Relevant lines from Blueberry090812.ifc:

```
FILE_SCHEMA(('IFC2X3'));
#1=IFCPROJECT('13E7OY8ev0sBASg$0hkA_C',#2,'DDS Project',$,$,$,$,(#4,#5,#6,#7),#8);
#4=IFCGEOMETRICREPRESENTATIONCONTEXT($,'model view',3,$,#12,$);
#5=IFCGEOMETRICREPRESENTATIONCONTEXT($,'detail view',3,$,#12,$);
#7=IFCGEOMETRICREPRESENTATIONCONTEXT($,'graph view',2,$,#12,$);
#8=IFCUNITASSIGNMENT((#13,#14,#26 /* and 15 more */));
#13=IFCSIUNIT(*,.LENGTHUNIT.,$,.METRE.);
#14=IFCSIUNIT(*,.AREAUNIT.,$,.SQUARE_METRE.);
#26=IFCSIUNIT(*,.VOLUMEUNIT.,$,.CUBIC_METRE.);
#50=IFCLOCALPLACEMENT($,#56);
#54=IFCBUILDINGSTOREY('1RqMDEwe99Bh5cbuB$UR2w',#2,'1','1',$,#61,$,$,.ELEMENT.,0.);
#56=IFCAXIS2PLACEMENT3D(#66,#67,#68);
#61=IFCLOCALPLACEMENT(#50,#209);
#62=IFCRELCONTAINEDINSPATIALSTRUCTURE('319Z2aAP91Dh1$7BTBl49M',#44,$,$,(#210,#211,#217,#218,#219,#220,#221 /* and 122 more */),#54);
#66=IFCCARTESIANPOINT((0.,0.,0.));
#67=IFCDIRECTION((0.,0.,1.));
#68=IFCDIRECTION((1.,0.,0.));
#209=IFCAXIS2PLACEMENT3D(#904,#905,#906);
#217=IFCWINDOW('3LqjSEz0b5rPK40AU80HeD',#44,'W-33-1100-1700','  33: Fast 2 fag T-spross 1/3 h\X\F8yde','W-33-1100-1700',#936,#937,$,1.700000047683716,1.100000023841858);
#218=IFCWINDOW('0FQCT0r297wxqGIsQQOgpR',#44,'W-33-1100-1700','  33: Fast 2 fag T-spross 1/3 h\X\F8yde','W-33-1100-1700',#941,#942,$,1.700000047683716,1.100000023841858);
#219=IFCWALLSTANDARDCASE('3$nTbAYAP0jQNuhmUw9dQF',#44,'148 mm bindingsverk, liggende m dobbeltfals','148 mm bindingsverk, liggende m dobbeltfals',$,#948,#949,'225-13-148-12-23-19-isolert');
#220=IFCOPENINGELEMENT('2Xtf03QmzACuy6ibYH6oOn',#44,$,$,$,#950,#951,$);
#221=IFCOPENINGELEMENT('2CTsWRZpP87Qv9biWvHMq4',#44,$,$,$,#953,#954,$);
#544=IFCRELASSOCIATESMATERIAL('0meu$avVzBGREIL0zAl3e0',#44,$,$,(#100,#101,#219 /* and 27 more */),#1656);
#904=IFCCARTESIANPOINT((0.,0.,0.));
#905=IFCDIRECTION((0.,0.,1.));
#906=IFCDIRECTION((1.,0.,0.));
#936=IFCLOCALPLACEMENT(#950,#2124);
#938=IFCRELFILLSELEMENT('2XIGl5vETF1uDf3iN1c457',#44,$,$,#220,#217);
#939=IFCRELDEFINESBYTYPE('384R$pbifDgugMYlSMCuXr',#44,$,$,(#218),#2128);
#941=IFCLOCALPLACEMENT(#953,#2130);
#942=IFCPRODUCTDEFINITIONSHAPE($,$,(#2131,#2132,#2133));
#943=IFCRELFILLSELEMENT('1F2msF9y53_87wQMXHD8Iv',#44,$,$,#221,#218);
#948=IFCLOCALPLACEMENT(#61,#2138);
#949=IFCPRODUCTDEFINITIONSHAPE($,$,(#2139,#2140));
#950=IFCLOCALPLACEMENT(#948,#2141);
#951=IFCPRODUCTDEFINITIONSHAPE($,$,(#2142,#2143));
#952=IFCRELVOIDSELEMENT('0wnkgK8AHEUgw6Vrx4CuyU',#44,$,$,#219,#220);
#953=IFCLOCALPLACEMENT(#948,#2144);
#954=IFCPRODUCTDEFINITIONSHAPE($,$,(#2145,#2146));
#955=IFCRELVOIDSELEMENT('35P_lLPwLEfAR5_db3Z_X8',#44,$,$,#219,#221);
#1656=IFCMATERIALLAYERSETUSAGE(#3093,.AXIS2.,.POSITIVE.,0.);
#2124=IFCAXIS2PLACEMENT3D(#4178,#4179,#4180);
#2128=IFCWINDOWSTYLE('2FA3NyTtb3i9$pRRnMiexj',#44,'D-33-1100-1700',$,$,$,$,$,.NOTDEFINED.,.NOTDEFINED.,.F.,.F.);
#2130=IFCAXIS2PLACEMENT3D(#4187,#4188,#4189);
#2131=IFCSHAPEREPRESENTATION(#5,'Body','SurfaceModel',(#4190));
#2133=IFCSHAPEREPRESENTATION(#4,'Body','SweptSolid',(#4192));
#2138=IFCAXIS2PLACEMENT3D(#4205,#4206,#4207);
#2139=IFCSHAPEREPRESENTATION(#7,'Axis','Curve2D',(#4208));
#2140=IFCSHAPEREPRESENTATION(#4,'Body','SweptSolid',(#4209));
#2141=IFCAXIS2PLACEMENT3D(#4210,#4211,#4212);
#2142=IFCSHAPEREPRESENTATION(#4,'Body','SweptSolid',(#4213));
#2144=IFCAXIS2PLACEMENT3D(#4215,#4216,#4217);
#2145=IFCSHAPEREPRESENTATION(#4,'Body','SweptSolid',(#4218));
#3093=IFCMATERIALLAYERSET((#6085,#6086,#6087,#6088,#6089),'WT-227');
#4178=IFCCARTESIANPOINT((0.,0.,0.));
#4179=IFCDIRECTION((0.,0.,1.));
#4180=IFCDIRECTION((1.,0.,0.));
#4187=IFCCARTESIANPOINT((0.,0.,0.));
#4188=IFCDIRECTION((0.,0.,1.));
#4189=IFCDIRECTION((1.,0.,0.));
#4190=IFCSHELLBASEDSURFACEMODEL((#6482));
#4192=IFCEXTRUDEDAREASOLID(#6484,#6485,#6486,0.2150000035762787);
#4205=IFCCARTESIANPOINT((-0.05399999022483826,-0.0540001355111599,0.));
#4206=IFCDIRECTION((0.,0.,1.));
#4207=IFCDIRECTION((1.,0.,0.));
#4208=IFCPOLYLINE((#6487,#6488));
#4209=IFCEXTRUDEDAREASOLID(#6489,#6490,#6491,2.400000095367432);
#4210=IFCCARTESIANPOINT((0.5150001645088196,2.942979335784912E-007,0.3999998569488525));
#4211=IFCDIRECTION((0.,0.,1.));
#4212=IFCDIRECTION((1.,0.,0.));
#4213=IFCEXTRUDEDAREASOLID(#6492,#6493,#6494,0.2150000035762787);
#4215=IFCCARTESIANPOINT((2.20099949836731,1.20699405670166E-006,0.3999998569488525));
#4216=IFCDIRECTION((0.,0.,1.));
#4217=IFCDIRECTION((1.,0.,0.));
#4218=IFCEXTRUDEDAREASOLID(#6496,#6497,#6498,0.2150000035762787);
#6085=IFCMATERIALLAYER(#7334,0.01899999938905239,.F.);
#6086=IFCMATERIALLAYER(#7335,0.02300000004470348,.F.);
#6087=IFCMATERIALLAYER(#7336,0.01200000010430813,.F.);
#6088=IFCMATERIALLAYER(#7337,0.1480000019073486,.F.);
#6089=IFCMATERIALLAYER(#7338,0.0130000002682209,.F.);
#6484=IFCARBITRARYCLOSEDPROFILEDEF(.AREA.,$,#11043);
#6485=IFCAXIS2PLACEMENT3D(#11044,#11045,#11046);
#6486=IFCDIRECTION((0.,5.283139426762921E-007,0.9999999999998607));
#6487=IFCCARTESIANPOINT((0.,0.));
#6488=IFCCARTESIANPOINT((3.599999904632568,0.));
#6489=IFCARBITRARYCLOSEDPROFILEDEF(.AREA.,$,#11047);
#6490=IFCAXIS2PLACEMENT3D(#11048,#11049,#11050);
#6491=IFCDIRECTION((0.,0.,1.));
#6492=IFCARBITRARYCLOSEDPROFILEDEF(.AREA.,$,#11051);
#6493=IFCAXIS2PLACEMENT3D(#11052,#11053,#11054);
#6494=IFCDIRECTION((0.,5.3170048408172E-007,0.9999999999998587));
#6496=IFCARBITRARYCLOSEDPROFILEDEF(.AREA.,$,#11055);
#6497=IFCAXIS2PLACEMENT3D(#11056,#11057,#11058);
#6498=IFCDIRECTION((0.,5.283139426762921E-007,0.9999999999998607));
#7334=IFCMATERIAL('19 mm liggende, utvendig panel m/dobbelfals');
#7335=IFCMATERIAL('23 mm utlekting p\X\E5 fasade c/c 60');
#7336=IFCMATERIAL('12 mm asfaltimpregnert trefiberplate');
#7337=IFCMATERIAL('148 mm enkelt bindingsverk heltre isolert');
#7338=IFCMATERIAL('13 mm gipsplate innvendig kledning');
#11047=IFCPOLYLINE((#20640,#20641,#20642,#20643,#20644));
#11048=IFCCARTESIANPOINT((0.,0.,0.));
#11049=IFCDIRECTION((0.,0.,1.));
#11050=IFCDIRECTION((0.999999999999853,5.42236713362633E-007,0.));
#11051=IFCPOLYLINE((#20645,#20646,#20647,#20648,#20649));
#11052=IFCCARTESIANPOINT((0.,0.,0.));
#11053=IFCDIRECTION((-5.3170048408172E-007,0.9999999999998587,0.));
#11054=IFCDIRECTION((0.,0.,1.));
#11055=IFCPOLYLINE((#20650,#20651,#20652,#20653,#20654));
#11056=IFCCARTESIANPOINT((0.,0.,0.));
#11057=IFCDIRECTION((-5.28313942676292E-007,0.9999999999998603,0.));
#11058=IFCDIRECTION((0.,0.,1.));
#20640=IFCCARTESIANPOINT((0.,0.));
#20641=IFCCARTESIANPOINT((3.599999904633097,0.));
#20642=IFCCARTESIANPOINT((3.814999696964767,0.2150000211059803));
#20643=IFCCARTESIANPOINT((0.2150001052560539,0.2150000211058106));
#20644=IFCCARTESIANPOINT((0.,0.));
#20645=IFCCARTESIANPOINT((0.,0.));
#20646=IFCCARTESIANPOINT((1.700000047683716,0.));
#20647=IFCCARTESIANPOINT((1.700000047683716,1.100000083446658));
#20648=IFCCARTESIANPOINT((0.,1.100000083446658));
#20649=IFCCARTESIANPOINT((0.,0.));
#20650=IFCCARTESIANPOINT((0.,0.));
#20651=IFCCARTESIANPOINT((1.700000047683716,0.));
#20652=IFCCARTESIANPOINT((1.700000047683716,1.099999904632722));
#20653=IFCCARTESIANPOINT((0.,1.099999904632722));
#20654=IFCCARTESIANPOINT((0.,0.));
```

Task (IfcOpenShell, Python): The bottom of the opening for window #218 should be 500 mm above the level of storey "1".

```python
import numpy as np
import ifcopenshell
import ifcopenshell.api.geometry
import ifcopenshell.geom
import ifcopenshell.util.element
import ifcopenshell.util.placement
import ifcopenshell.util.shape
import ifcopenshell.util.unit

model = ifcopenshell.open("Blueberry090812.ifc")
unit_scale = ifcopenshell.util.unit.calculate_unit_scale(model)

window = model.by_guid("0FQCT0r297wxqGIsQQOgpR")
opening = window.FillsVoids[0].RelatingOpeningElement
storey = ifcopenshell.util.element.get_container(window, ifc_class="IfcBuildingStorey")
level = ifcopenshell.util.placement.get_local_placement(storey.ObjectPlacement)[2, 3]

# The opening's origin need not be at the sill, so measure its lowest point.
shape = ifcopenshell.geom.create_shape(ifcopenshell.geom.settings(), opening)
bottom = ifcopenshell.util.shape.get_shape_bottom_elevation(shape, shape.geometry) / unit_scale
dz = level + 0.5 - bottom

shift = np.array([0.0, 0.0, dz])
# The window is placed relative to its opening, so it follows when the opening moves.
matrix = ifcopenshell.util.placement.get_local_placement(opening.ObjectPlacement)
matrix[:3, 3] += shift
ifcopenshell.api.geometry.edit_object_placement(
    model, product=opening, matrix=matrix, is_si=False, should_transform_children=True
)

print(f"moved by {dz * unit_scale:+.3f} m")

model.write("Blueberry090812_updated.ifc")
```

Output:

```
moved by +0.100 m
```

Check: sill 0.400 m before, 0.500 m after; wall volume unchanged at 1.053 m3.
